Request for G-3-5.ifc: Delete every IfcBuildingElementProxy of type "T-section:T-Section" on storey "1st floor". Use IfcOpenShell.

First a look at what the model holds.

```python
import ifcopenshell
import ifcopenshell.util.element

model = ifcopenshell.open("G-3-5.ifc")
print(model.schema)
storey = next(s for s in model.by_type("IfcBuildingStorey") if s.Name == "1st floor")
proxies = [e for e in ifcopenshell.util.element.get_decomposition(storey) if e.is_a("IfcBuildingElementProxy")]
seen = {}
for e in proxies:
    element_type = ifcopenshell.util.element.get_type(e)
    name = element_type.Name if element_type not in (None, e) else None
    seen[name] = seen.get(name, 0) + 1
for name, count in sorted(seen.items(), key=str):
    print(count, "x", name)
```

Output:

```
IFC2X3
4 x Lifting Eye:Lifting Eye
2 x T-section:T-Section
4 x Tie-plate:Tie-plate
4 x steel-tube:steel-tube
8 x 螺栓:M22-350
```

```python
import ifcopenshell
import ifcopenshell.api.root
import ifcopenshell.util.element

model = ifcopenshell.open("G-3-5.ifc")

storey = next(s for s in model.by_type("IfcBuildingStorey") if s.Name == "1st floor")
proxies = [e for e in ifcopenshell.util.element.get_decomposition(storey) if e.is_a("IfcBuildingElementProxy")]
targets = [e for e in proxies if (t := ifcopenshell.util.element.get_type(e)) not in (None, e) and t.Name == "T-section:T-Section"]

for e in targets:
    ifcopenshell.api.root.remove_product(model, product=e)
print(len(targets), "removed")

model.write("G-3-5_updated.ifc")
```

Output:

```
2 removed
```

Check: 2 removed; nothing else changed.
